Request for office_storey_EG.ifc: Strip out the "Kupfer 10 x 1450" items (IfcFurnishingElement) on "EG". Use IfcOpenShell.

First a look at what the model holds.

```python
import ifcopenshell
import ifcopenshell.util.element

model = ifcopenshell.open("office_storey_EG.ifc")
print(model.schema)
storey = next(s for s in model.by_type("IfcBuildingStorey") if s.Name == "EG")
furniture = [e for e in ifcopenshell.util.element.get_decomposition(storey) if e.is_a("IfcFurnishingElement")]
seen = {}
for e in furniture:
    element_type = ifcopenshell.util.element.get_type(e)
    name = element_type.Name if element_type not in (None, e) else None
    seen[name] = seen.get(name, 0) + 1
for name, count in sorted(seen.items(), key=str):
    print(count, "x", name)
```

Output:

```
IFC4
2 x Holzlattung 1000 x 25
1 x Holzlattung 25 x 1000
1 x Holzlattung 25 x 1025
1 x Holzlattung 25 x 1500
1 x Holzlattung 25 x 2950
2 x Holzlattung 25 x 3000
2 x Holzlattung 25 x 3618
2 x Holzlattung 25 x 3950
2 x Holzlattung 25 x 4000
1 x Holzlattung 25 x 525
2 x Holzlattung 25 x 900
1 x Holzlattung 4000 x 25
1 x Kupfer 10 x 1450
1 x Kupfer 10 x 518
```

```python
import ifcopenshell
import ifcopenshell.api.root
import ifcopenshell.util.element

model = ifcopenshell.open("office_storey_EG.ifc")

storey = next(s for s in model.by_type("IfcBuildingStorey") if s.Name == "EG")
furniture = [e for e in ifcopenshell.util.element.get_decomposition(storey) if e.is_a("IfcFurnishingElement")]
targets = [e for e in furniture if (t := ifcopenshell.util.element.get_type(e)) not in (None, e) and t.Name == "Kupfer 10 x 1450"]

for e in targets:
    ifcopenshell.api.root.remove_product(model, product=e)
print(len(targets), "removed")

model.write("office_storey_EG-out.ifc")
```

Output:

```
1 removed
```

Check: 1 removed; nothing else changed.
